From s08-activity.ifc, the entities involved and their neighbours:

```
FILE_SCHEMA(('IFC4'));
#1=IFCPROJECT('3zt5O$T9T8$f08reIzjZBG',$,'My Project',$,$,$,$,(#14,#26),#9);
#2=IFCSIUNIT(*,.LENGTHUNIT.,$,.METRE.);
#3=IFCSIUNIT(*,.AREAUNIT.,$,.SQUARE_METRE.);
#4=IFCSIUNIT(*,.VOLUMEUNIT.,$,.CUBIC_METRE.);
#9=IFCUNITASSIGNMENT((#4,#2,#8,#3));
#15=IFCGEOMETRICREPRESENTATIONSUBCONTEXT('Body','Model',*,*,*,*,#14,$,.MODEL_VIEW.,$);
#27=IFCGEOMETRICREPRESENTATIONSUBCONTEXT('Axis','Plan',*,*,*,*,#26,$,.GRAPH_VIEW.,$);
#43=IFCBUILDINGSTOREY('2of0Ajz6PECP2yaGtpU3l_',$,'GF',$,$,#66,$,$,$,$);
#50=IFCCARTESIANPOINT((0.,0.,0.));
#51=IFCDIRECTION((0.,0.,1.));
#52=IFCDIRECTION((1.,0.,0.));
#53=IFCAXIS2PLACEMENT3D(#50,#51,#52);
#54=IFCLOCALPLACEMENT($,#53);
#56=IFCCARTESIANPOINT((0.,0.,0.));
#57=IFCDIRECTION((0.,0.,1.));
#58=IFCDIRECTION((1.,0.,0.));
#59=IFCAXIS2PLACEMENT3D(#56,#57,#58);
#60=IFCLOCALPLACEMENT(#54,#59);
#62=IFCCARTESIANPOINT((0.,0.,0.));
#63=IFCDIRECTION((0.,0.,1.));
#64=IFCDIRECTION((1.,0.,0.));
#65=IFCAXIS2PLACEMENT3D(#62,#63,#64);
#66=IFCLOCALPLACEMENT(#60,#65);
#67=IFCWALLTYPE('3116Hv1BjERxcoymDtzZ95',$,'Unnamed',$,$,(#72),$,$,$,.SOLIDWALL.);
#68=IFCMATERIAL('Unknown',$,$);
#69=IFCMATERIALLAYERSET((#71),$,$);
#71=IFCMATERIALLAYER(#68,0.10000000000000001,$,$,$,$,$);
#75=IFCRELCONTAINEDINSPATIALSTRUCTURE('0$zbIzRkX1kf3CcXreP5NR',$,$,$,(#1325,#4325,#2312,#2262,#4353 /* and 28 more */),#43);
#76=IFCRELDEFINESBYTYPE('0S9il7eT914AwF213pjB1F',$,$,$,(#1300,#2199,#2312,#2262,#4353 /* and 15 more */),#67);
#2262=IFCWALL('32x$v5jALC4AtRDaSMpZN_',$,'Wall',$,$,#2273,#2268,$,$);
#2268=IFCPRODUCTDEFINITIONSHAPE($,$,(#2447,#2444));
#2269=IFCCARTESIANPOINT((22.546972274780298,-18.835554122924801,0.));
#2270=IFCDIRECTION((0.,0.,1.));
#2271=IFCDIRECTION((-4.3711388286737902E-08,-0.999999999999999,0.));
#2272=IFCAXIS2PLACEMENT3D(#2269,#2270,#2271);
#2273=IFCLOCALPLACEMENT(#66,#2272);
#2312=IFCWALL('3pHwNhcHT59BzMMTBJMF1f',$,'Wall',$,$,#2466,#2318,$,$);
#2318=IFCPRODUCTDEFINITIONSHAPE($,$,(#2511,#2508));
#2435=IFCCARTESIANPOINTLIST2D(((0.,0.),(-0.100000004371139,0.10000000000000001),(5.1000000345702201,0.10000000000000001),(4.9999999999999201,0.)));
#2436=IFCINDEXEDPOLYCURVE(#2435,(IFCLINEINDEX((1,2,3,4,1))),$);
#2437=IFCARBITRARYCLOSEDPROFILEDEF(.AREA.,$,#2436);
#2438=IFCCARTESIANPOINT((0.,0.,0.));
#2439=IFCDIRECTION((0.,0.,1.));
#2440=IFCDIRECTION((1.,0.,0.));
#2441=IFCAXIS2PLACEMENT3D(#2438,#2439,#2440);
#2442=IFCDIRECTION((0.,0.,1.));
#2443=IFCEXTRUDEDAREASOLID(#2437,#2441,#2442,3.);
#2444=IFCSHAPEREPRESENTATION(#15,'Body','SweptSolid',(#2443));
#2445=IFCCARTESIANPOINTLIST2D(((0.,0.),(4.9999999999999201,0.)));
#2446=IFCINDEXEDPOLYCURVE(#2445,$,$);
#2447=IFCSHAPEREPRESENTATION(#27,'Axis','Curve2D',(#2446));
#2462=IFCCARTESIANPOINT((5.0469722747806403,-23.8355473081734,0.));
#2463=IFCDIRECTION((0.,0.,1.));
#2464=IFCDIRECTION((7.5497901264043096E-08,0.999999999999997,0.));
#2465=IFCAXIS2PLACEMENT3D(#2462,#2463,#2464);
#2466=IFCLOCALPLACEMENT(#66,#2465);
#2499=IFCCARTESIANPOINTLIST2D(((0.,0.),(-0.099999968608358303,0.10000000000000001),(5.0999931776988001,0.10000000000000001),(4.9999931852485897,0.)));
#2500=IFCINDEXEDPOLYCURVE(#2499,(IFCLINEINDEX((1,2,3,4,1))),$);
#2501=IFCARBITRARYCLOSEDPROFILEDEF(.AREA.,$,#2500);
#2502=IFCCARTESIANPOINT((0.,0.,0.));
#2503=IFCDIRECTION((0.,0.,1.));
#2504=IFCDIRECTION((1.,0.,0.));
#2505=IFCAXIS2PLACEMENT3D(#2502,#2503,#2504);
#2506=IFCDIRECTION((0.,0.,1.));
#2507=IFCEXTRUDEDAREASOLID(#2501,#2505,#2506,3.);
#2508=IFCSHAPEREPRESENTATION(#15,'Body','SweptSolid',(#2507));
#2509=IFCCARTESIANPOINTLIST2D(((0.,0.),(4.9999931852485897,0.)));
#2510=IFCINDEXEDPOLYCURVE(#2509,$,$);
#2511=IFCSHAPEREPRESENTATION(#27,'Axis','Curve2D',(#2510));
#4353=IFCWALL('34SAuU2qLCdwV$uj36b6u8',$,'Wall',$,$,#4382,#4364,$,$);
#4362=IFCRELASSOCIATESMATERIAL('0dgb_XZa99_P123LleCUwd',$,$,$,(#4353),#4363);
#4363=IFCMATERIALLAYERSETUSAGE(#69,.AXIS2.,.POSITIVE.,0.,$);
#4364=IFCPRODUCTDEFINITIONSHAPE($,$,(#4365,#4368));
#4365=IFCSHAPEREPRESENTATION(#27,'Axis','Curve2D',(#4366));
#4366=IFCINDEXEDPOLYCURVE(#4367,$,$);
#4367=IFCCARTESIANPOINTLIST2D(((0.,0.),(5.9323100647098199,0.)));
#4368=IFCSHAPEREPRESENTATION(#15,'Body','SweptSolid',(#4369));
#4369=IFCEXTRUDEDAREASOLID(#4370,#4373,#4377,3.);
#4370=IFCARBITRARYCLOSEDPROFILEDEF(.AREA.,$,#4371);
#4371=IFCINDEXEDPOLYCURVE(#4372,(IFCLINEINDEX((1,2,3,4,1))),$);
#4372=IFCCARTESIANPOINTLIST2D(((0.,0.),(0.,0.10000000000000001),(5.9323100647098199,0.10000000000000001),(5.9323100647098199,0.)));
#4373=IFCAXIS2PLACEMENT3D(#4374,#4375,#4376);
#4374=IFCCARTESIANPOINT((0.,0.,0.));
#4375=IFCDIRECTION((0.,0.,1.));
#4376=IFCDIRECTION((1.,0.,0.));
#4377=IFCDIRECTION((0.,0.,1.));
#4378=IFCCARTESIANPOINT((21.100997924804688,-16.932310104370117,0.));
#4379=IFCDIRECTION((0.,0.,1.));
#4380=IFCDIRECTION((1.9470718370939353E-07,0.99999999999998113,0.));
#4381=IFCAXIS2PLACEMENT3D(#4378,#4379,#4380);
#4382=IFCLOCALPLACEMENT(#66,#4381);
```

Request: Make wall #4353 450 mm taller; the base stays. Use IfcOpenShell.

```python
import ifcopenshell
import ifcopenshell.geom
import ifcopenshell.util.representation
import ifcopenshell.util.shape

model = ifcopenshell.open("s08-activity.ifc")
settings = ifcopenshell.geom.settings()


def volume(element):
    """Net volume in cubic metres, openings subtracted."""
    shape = ifcopenshell.geom.create_shape(settings, element)
    return ifcopenshell.util.shape.get_volume(shape.geometry)


wall = model.by_guid("34SAuU2qLCdwV$uj36b6u8")
before = volume(wall)

body = ifcopenshell.util.representation.get_representation(wall, "Model", "Body")
solid = body.Items[0]
old_height = solid.Depth
solid.Depth += 0.45
after = volume(wall)

print(f"height {old_height:g} -> {solid.Depth:g}, volume {before:.3f} -> {after:.3f} m3")

model.write("s08-activity-out.ifc")
```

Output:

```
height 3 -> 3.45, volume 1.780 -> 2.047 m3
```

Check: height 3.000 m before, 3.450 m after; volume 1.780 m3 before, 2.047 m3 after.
